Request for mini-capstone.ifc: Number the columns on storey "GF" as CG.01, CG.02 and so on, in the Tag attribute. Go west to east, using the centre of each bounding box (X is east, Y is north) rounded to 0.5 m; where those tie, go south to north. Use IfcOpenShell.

First a look at what the model holds.

```python
import ifcopenshell
import ifcopenshell.util.element
import ifcopenshell.util.placement

model = ifcopenshell.open("mini-capstone.ifc")
print(model.schema)
storey = next(s for s in model.by_type("IfcBuildingStorey") if s.Name == "GF")
columns = [e for e in ifcopenshell.util.element.get_decomposition(storey) if e.is_a("IfcColumn")]
for e in sorted(columns, key=lambda e: e.id()):
    origin = ifcopenshell.util.placement.get_local_placement(e.ObjectPlacement)[:3, 3]
    print(e.id(), e.Tag, e.Name, origin.round(2) + 0.0, sep=" | ")
```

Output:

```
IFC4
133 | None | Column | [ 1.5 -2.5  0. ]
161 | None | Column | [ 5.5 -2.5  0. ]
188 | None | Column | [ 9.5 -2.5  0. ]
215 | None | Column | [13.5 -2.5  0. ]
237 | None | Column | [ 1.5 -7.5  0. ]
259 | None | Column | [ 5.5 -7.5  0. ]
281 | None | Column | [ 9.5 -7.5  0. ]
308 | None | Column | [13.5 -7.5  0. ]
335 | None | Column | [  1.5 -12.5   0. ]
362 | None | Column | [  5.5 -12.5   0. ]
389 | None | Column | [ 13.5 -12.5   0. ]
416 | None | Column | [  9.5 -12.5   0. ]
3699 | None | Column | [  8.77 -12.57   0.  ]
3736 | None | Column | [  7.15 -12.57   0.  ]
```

```python
import ifcopenshell
import ifcopenshell.geom
import ifcopenshell.util.element
import ifcopenshell.util.shape

model = ifcopenshell.open("mini-capstone.ifc")
settings = ifcopenshell.geom.settings()
settings.set("use-world-coords", True)


def centre(element):
    shape = ifcopenshell.geom.create_shape(settings, element)
    return ifcopenshell.util.shape.get_bbox_centroid(shape.geometry)


storey = next(s for s in model.by_type("IfcBuildingStorey") if s.Name == "GF")
columns = [e for e in ifcopenshell.util.element.get_decomposition(storey) if e.is_a("IfcColumn")]

# Insertion points can sit at a corner or the storey origin, so sort by the geometry (in metres).
centres = {e: centre(e) for e in columns}
columns.sort(key=lambda e: (round(centres[e][0] / 0.5), centres[e][1]))

for i, e in enumerate(columns, start=1):
    number = f"CG.{i:02d}"
    e.Tag = number
    print(e.id(), number)

model.write("mini-capstone_edited.ifc")
```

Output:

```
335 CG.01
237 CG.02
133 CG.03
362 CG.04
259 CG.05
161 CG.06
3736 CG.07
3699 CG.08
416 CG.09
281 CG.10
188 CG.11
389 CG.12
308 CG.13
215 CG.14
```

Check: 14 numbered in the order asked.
